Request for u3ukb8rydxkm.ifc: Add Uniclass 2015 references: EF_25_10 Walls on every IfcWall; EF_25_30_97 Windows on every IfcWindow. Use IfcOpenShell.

First a look at what the model holds.

```python
import ifcopenshell

model = ifcopenshell.open("u3ukb8rydxkm.ifc")
print(model.schema)
print("classifications:", [c.Name for c in model.by_type("IfcClassification")])
for ifc_class in ("IfcDoor", "IfcRoof", "IfcStair", "IfcWall", "IfcWindow"):
    print(ifc_class, len(model.by_type(ifc_class)))
```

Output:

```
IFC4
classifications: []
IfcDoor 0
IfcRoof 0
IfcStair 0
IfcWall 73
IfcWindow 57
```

```python
import ifcopenshell
import ifcopenshell.api.classification

model = ifcopenshell.open("u3ukb8rydxkm.ifc")

system = ifcopenshell.api.classification.add_classification(model, classification="Uniclass 2015")

codes = {
    "IfcWall": ("EF_25_10", "Walls"),
    "IfcWindow": ("EF_25_30_97", "Windows"),
}
for ifc_class, (code, name) in codes.items():
    products = model.by_type(ifc_class)
    ifcopenshell.api.classification.add_reference(
        model, products=products, classification=system, identification=code, name=name
    )
    print(code, len(products))

model.write("u3ukb8rydxkm_rev.ifc")
```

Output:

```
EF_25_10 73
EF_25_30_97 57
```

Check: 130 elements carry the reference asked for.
